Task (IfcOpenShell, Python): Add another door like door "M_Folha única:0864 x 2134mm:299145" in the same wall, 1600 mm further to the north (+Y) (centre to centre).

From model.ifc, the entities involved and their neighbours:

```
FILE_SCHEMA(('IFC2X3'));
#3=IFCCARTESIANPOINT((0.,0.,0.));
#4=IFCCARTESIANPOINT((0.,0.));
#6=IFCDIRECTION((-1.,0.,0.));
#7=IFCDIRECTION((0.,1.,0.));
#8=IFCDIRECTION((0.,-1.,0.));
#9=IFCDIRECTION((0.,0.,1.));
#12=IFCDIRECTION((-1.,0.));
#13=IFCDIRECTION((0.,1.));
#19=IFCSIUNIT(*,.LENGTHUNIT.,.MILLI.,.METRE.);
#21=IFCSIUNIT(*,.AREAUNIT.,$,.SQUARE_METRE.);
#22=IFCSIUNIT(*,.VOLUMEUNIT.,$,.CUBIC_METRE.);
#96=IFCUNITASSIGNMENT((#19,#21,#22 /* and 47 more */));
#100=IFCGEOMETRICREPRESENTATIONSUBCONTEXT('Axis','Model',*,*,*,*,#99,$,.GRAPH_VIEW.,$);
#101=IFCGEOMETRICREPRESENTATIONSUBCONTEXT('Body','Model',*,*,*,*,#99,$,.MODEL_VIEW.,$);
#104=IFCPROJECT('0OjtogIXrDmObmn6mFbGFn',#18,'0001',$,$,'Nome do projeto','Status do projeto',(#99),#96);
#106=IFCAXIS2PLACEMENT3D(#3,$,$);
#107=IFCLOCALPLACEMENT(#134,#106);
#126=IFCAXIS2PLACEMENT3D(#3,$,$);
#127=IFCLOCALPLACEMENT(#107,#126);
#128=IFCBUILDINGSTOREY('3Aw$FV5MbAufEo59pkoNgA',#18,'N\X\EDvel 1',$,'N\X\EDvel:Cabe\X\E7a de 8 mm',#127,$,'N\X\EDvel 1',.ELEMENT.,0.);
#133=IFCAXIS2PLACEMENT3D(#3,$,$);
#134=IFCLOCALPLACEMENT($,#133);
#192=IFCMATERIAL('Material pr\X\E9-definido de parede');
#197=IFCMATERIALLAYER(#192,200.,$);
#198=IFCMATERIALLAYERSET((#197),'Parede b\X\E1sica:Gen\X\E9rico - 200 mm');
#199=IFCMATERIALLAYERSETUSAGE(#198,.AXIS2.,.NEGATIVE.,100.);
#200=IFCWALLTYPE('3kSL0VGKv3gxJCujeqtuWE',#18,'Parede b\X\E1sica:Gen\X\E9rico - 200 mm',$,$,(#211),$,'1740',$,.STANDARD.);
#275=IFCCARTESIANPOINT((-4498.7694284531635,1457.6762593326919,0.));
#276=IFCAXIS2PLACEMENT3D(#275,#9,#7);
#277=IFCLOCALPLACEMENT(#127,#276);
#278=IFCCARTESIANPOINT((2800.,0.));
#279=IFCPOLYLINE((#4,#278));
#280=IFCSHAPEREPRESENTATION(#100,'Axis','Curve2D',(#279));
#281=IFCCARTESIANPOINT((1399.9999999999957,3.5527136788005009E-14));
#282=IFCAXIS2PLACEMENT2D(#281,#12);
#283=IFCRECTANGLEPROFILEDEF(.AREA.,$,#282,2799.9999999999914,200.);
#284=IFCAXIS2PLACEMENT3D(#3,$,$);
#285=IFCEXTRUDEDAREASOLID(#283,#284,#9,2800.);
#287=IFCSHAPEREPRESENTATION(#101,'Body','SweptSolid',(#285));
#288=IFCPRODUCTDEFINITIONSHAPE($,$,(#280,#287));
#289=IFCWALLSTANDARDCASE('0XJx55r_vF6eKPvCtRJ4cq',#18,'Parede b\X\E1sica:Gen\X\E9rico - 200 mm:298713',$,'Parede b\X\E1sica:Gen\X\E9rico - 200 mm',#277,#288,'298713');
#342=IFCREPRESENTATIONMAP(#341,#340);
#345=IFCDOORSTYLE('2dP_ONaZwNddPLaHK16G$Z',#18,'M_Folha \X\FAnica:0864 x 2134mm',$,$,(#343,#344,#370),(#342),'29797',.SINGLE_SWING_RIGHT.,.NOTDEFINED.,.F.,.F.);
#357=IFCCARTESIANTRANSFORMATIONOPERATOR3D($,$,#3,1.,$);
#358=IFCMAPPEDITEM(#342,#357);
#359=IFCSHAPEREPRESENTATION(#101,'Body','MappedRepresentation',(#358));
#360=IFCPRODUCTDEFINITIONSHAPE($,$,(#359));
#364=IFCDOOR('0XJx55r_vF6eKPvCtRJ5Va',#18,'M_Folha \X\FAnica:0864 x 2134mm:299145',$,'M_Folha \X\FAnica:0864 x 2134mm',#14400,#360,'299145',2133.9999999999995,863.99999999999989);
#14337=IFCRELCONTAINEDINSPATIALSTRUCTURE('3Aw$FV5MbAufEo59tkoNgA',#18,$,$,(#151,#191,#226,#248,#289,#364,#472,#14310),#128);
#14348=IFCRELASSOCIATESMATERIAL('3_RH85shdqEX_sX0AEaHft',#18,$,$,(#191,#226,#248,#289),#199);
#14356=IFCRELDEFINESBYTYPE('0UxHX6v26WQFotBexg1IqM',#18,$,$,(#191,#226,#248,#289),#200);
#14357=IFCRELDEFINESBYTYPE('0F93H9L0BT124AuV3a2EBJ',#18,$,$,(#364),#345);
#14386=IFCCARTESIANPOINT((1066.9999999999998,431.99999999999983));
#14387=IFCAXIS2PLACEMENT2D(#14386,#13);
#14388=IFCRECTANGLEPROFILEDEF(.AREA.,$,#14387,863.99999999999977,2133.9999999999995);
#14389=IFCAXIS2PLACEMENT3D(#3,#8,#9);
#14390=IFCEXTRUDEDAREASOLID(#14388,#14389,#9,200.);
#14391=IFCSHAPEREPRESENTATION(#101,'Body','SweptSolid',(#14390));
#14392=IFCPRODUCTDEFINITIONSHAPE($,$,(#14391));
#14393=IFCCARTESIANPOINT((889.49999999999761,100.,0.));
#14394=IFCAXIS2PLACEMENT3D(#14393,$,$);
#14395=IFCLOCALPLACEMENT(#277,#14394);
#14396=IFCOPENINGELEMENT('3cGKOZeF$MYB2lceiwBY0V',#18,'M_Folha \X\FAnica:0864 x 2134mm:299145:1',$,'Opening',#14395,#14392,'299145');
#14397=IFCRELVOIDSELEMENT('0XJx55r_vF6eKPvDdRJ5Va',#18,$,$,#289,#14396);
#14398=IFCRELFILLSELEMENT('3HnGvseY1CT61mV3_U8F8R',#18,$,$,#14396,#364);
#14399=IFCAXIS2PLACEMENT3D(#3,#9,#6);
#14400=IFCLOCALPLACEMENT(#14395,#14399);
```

```python
import ifcopenshell
import ifcopenshell.api.feature
import ifcopenshell.api.geometry
import ifcopenshell.api.root
import ifcopenshell.geom
import ifcopenshell.util.element
import ifcopenshell.util.placement
import ifcopenshell.util.shape
import ifcopenshell.util.unit

model = ifcopenshell.open("model.ifc")
unit_scale = ifcopenshell.util.unit.calculate_unit_scale(model)
settings = ifcopenshell.geom.settings()


def volume(element):
    """Net volume in cubic metres, openings subtracted."""
    shape = ifcopenshell.geom.create_shape(settings, element)
    return ifcopenshell.util.shape.get_volume(shape.geometry)


def reuse_history(source, copy):
    """copy_class also copies each property set's owner history, people and application; keep the originals."""
    for rel in copy.IsDefinedBy:
        if rel.is_a("IfcRelDefinesByProperties") and (history := rel.RelatingPropertyDefinition.OwnerHistory):
            rel.RelatingPropertyDefinition.OwnerHistory = source.OwnerHistory
            ifcopenshell.util.element.remove_deep2(model, history)


door = model.by_guid("0XJx55r_vF6eKPvCtRJ5Va")
opening = door.FillsVoids[0].RelatingOpeningElement
wall = opening.VoidsElements[0].RelatingBuildingElement
before = volume(wall)
shift = ifcopenshell.util.placement.get_local_placement(wall.ObjectPlacement)[:3, 0] * 1.6 / unit_scale

# copy_class copies the void relationship, type, container and properties, but no geometry.
new_opening = ifcopenshell.api.root.copy_class(model, product=opening)
new_opening.Representation = ifcopenshell.util.element.copy_deep(
    model, opening.Representation, exclude=["IfcGeometricRepresentationContext", "IfcRepresentationMap"]
)
new_opening.Name = "M_Folha única:0864 x 2134mm"
new_opening.Tag = None
new_door = ifcopenshell.api.root.copy_class(model, product=door)
new_door.Representation = ifcopenshell.util.element.copy_deep(
    model, door.Representation, exclude=["IfcGeometricRepresentationContext", "IfcRepresentationMap"]
)
new_door.Name = "M_Folha única:0864 x 2134mm"
new_door.Tag = None
reuse_history(door, new_door)
fills = ifcopenshell.api.feature.add_filling(model, opening=new_opening, element=new_door)
fills.OwnerHistory = new_door.OwnerHistory  # required in IFC2X3

for old, new in ((opening, new_opening), (door, new_door)):
    matrix = ifcopenshell.util.placement.get_local_placement(old.ObjectPlacement)
    matrix[:3, 3] += shift
    ifcopenshell.api.geometry.edit_object_placement(model, product=new, matrix=matrix, is_si=False)

after = volume(wall)

print(f"wall volume {before:.3f} -> {after:.3f} m3")

model.write("model_rev.ifc")
```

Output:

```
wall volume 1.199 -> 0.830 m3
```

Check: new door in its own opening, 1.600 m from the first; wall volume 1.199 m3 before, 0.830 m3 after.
